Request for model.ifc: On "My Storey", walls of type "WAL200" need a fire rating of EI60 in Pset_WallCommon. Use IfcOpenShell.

First a look at what the model holds.

```python
import ifcopenshell
import ifcopenshell.util.element

model = ifcopenshell.open("model.ifc")
print(model.schema)
storey = next(s for s in model.by_type("IfcBuildingStorey") if s.Name == "My Storey")
walls = [e for e in ifcopenshell.util.element.get_decomposition(storey) if e.is_a("IfcWall")]
seen = {}
for e in walls:
    element_type = ifcopenshell.util.element.get_type(e)
    key = (element_type.Name if element_type != e and element_type else None, ifcopenshell.util.element.get_pset(e, "Pset_WallCommon", "FireRating"))
    seen[key] = seen.get(key, 0) + 1
for (name, value), count in sorted(seen.items(), key=str):
    print(count, "x", name, "|", value)
```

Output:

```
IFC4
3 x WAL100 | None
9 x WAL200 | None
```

```python
import ifcopenshell
import ifcopenshell.api.pset
import ifcopenshell.util.element

model = ifcopenshell.open("model.ifc")

storey = next(s for s in model.by_type("IfcBuildingStorey") if s.Name == "My Storey")
walls = [e for e in ifcopenshell.util.element.get_decomposition(storey) if e.is_a("IfcWall")]

count = 0
for e in walls:
    element_type = ifcopenshell.util.element.get_type(e)
    if element_type in (None, e) or element_type.Name != "WAL200":
        continue
    # add_pset returns the element's existing set when there is one.
    pset = ifcopenshell.api.pset.add_pset(model, product=e, name="Pset_WallCommon")
    ifcopenshell.api.pset.edit_pset(model, pset=pset, properties={"FireRating": "EI60"})
    count += 1

print(count, "walls updated")

model.write("model_edited.ifc")
```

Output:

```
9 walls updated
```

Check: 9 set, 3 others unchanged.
